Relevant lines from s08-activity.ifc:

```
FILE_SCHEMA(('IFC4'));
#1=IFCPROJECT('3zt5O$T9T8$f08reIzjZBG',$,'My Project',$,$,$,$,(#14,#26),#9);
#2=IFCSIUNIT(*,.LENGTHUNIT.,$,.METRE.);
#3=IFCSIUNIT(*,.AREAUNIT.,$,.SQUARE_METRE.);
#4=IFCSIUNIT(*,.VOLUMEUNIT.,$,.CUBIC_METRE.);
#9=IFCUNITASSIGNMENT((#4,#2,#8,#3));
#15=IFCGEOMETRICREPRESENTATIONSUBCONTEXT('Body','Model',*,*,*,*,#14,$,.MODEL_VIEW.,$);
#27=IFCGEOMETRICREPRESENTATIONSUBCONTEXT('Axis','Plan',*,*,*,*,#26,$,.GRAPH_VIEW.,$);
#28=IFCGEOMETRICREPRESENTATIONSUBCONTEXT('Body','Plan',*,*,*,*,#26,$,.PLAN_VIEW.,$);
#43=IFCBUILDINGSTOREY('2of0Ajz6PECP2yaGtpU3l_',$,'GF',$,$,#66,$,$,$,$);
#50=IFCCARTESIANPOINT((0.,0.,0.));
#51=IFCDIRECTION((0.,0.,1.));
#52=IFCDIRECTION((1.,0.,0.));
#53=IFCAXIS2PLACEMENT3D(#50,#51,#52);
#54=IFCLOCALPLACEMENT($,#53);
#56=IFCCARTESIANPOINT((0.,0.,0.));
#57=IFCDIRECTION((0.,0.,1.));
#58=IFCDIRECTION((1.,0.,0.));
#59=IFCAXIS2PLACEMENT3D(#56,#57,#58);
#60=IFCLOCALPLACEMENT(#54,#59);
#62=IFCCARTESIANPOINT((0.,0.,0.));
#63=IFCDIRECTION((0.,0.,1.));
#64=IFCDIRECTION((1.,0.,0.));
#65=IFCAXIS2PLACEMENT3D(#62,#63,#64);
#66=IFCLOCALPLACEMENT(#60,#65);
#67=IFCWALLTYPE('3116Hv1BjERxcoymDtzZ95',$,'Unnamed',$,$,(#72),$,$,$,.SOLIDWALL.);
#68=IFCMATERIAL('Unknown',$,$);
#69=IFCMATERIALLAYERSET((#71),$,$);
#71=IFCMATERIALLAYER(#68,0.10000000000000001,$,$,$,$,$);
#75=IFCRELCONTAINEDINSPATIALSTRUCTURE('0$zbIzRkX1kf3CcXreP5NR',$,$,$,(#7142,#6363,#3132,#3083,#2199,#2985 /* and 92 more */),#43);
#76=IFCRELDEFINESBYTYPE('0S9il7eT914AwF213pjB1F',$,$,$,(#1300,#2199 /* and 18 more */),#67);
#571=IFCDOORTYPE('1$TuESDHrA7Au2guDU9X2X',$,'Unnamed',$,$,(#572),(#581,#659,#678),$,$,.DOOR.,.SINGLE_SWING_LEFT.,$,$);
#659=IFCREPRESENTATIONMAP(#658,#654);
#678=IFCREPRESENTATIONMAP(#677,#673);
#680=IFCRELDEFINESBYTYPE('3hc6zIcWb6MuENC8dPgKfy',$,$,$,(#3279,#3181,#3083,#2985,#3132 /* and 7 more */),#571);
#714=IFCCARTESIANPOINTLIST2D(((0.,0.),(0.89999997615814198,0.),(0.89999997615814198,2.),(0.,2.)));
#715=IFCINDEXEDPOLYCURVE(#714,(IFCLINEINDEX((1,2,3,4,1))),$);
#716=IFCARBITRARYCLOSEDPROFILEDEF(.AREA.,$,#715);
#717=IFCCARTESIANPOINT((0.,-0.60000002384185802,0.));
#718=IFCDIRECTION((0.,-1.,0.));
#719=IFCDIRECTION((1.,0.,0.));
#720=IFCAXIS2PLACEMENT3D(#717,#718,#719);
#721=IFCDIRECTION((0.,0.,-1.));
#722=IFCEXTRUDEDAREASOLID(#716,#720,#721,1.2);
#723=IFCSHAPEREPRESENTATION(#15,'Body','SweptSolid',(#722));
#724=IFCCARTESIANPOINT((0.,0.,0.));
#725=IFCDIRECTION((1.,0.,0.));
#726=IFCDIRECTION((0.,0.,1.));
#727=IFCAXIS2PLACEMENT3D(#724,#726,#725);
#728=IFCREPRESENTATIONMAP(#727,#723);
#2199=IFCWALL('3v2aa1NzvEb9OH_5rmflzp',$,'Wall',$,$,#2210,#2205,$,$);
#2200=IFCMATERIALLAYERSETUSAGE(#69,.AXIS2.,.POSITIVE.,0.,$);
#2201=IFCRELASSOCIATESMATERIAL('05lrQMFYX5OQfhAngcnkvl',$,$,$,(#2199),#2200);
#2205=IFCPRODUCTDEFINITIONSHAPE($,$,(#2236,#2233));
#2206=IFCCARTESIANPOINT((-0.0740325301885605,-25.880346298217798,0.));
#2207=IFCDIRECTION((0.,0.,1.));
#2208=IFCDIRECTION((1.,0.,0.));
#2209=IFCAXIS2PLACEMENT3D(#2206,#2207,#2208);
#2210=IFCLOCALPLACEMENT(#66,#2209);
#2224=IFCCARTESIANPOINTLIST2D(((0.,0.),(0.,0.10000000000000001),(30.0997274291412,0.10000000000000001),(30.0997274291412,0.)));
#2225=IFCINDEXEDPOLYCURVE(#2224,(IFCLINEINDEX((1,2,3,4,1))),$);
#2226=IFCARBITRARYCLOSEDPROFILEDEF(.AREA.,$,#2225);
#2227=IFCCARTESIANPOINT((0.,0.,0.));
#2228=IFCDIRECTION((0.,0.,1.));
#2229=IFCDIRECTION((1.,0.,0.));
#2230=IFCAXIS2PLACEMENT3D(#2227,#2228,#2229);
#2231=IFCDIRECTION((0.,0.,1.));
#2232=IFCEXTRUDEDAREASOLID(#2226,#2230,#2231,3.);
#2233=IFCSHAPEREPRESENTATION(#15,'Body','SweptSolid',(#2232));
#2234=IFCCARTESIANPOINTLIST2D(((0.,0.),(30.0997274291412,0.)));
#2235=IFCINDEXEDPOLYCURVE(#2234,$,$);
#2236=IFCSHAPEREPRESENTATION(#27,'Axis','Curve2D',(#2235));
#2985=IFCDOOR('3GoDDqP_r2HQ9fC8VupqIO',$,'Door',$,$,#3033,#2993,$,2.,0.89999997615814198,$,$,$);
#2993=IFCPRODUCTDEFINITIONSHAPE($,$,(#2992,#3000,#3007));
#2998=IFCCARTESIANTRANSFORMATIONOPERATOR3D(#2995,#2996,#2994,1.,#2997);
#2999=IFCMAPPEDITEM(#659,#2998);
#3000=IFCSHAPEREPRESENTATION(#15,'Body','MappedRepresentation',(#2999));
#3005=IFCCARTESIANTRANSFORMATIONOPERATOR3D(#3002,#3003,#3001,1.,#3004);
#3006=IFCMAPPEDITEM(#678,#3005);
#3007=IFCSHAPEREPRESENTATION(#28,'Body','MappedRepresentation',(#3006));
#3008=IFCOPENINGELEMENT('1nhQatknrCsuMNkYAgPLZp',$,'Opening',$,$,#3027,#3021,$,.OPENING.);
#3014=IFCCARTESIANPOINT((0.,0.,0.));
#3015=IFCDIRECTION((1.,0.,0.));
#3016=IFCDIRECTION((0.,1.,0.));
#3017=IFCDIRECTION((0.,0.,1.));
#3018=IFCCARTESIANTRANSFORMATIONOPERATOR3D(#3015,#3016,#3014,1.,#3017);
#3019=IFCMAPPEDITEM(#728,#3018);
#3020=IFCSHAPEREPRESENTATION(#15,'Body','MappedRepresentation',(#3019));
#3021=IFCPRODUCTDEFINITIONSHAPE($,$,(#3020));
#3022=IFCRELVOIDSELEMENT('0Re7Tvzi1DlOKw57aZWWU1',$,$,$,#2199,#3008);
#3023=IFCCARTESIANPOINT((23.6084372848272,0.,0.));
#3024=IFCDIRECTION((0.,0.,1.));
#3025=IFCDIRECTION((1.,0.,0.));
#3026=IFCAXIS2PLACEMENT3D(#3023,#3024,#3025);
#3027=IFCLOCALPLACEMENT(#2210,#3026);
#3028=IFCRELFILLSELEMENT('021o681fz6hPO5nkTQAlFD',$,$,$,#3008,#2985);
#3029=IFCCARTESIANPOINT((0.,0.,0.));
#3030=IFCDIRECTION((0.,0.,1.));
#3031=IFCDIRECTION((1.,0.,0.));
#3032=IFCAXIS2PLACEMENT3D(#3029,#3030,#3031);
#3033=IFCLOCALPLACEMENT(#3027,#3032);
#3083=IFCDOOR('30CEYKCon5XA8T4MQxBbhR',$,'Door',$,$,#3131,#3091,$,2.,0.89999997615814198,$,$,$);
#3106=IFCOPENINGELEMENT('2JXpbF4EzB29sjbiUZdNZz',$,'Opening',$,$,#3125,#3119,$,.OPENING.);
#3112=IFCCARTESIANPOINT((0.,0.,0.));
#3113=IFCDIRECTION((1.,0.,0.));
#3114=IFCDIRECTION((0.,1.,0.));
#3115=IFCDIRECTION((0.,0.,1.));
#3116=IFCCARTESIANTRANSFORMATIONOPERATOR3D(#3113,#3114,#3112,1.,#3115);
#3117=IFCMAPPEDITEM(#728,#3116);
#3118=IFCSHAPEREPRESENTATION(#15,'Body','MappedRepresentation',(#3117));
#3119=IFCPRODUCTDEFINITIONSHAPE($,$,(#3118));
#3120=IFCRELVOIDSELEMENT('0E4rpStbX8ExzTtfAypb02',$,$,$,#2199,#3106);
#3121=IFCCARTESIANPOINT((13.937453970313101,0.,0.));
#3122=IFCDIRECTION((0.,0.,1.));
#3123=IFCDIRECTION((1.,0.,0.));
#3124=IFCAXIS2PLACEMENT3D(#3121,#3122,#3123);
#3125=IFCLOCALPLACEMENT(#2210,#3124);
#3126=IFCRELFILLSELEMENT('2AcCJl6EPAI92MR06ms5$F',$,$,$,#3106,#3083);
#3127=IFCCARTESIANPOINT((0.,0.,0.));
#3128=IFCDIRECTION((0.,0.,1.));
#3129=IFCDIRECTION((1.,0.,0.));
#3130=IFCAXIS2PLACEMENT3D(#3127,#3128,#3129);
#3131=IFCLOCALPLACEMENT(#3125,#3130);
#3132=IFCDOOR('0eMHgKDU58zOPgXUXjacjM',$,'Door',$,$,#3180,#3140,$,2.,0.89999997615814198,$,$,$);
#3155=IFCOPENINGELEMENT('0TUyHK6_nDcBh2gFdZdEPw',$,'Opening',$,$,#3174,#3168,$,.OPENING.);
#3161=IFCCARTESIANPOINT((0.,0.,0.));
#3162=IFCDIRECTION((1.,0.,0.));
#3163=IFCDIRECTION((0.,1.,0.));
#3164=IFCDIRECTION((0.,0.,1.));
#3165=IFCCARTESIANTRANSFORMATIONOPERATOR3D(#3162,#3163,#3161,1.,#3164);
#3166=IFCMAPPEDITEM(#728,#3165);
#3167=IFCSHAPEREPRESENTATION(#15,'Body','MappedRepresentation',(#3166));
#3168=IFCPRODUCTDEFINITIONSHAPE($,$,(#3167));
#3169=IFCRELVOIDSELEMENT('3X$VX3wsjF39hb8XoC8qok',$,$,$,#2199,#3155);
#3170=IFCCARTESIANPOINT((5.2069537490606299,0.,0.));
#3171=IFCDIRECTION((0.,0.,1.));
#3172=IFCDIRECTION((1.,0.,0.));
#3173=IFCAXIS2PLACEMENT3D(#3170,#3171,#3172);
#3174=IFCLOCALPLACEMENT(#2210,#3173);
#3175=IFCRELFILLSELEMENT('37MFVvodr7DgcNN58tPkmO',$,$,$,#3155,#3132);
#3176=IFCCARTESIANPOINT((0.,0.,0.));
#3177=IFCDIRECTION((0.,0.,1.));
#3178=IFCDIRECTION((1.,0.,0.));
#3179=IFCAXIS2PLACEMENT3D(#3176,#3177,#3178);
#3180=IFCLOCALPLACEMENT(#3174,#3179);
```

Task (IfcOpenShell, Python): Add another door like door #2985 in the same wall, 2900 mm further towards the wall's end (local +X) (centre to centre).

```python
import ifcopenshell
import ifcopenshell.api.feature
import ifcopenshell.api.geometry
import ifcopenshell.api.root
import ifcopenshell.geom
import ifcopenshell.util.element
import ifcopenshell.util.placement
import ifcopenshell.util.shape
import ifcopenshell.util.unit

model = ifcopenshell.open("s08-activity.ifc")
unit_scale = ifcopenshell.util.unit.calculate_unit_scale(model)
settings = ifcopenshell.geom.settings()


def volume(element):
    """Net volume in cubic metres, openings subtracted."""
    shape = ifcopenshell.geom.create_shape(settings, element)
    return ifcopenshell.util.shape.get_volume(shape.geometry)


door = model.by_id(2985)
opening = door.FillsVoids[0].RelatingOpeningElement
wall = opening.VoidsElements[0].RelatingBuildingElement
before = volume(wall)
shift = ifcopenshell.util.placement.get_local_placement(wall.ObjectPlacement)[:3, 0] * 2.9 / unit_scale

# copy_class copies the void relationship, type, container and properties, but no geometry.
new_opening = ifcopenshell.api.root.copy_class(model, product=opening)
new_opening.Representation = ifcopenshell.util.element.copy_deep(
    model, opening.Representation, exclude=["IfcGeometricRepresentationContext", "IfcRepresentationMap"]
)
new_door = ifcopenshell.api.root.copy_class(model, product=door)
new_door.Representation = ifcopenshell.util.element.copy_deep(
    model, door.Representation, exclude=["IfcGeometricRepresentationContext", "IfcRepresentationMap"]
)
ifcopenshell.api.feature.add_filling(model, opening=new_opening, element=new_door)

for old, new in ((opening, new_opening), (door, new_door)):
    matrix = ifcopenshell.util.placement.get_local_placement(old.ObjectPlacement)
    matrix[:3, 3] += shift
    ifcopenshell.api.geometry.edit_object_placement(model, product=new, matrix=matrix, is_si=False)

after = volume(wall)

print(f"wall volume {before:.3f} -> {after:.3f} m3")

model.write("s08-activity_v2.ifc")
```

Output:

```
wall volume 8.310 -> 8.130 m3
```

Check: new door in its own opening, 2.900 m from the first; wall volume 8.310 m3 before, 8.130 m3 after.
